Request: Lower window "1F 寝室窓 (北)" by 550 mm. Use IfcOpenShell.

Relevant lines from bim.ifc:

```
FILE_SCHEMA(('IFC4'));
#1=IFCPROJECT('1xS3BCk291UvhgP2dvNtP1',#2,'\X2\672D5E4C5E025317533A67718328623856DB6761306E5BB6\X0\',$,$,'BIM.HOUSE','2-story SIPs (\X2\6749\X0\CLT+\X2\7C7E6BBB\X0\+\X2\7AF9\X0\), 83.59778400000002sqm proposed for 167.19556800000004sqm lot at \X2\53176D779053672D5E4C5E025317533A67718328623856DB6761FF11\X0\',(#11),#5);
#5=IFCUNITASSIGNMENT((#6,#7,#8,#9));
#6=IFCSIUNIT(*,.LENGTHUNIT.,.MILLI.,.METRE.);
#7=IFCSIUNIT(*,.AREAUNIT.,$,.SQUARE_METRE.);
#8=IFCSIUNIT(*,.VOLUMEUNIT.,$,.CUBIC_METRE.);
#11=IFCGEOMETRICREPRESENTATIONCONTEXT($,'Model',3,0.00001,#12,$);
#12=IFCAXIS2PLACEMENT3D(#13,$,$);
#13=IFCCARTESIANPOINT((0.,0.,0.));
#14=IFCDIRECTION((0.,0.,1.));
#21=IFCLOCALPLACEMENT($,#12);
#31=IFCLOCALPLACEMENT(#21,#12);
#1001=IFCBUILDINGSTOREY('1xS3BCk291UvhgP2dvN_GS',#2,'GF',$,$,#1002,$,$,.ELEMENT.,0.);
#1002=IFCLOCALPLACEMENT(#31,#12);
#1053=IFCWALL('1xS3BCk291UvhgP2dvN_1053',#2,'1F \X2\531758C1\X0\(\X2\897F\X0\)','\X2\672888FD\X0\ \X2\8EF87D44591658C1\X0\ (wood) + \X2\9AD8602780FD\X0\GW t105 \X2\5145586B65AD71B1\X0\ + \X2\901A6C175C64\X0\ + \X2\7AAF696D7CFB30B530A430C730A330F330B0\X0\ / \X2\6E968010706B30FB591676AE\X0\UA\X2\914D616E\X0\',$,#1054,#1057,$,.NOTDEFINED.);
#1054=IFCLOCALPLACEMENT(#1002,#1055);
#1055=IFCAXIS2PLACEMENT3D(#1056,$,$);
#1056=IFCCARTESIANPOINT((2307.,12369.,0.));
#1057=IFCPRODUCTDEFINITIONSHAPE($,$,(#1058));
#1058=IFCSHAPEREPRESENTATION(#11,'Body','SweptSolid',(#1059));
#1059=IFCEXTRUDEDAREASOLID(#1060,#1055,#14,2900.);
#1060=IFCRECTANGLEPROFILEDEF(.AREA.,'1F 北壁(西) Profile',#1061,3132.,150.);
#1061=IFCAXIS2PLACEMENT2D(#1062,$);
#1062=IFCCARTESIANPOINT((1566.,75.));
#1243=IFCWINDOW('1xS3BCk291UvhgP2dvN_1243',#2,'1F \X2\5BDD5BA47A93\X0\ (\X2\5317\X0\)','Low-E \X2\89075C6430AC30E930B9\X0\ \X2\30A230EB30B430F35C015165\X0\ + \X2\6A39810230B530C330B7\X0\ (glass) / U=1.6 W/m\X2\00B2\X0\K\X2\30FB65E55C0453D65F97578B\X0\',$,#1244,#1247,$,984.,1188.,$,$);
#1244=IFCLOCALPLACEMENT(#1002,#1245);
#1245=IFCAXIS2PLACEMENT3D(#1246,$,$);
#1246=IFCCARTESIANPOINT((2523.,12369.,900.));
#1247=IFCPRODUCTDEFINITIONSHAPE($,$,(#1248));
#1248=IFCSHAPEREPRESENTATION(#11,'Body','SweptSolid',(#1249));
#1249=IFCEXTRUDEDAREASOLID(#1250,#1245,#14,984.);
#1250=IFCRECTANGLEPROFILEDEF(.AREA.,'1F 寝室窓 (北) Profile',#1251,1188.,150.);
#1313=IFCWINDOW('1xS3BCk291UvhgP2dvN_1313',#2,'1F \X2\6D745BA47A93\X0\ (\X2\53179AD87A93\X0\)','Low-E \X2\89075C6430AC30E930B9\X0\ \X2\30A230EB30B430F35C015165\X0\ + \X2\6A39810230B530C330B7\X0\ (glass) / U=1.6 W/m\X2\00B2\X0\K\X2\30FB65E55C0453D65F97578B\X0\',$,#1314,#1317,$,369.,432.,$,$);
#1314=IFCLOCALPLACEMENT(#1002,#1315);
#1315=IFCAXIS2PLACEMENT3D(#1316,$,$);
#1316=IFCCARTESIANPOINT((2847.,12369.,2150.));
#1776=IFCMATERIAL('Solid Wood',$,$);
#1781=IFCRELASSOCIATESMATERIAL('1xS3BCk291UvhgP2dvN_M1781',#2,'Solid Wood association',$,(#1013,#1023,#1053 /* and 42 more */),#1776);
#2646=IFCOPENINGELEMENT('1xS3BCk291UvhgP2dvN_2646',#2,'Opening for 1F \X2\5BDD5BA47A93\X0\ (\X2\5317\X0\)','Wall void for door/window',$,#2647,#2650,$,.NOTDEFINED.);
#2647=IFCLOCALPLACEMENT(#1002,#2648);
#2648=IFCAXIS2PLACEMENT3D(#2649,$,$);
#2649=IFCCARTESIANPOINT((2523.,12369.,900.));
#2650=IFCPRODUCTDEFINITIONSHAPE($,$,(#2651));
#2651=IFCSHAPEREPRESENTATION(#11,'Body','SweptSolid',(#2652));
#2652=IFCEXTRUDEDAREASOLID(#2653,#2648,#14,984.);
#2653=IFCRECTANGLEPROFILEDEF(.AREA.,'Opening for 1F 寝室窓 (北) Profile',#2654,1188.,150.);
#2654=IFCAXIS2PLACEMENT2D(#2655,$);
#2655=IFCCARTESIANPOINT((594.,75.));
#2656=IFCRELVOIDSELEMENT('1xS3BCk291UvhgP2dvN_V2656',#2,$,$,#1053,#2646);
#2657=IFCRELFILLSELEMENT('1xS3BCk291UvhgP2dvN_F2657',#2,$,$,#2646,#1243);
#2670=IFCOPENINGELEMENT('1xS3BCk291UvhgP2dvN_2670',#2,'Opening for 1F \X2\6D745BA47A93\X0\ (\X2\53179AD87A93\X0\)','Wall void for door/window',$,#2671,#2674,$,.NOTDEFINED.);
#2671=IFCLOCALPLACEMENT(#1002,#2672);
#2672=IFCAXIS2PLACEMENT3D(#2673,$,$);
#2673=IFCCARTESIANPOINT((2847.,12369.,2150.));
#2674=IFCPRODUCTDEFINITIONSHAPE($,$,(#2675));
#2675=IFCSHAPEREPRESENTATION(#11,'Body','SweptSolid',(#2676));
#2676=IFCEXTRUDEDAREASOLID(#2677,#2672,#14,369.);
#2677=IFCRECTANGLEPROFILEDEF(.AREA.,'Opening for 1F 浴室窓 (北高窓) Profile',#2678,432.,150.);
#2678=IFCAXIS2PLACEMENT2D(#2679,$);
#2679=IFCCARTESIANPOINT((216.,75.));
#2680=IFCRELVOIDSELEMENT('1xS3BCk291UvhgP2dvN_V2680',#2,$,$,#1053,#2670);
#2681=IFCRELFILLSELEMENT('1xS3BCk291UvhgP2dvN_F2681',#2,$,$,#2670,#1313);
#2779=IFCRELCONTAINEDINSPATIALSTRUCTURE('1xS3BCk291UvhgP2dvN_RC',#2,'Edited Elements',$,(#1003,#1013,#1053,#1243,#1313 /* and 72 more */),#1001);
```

```python
import numpy as np
import ifcopenshell
import ifcopenshell.api.geometry
import ifcopenshell.util.placement
import ifcopenshell.util.unit

model = ifcopenshell.open("bim.ifc")
unit_scale = ifcopenshell.util.unit.calculate_unit_scale(model)

window = model.by_guid("1xS3BCk291UvhgP2dvN_1243")
opening = window.FillsVoids[0].RelatingOpeningElement
dz = -550.0

shift = np.array([0.0, 0.0, dz])
# The window is not placed relative to its opening, so move both.
for product in (opening, window):
    matrix = ifcopenshell.util.placement.get_local_placement(product.ObjectPlacement)
    matrix[:3, 3] += shift
    ifcopenshell.api.geometry.edit_object_placement(model, product=product, matrix=matrix, is_si=False)

print(f"moved by {dz * unit_scale:+.3f} m")

model.write("bim_edited.ifc")
```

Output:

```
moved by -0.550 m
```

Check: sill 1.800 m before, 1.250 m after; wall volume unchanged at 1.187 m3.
